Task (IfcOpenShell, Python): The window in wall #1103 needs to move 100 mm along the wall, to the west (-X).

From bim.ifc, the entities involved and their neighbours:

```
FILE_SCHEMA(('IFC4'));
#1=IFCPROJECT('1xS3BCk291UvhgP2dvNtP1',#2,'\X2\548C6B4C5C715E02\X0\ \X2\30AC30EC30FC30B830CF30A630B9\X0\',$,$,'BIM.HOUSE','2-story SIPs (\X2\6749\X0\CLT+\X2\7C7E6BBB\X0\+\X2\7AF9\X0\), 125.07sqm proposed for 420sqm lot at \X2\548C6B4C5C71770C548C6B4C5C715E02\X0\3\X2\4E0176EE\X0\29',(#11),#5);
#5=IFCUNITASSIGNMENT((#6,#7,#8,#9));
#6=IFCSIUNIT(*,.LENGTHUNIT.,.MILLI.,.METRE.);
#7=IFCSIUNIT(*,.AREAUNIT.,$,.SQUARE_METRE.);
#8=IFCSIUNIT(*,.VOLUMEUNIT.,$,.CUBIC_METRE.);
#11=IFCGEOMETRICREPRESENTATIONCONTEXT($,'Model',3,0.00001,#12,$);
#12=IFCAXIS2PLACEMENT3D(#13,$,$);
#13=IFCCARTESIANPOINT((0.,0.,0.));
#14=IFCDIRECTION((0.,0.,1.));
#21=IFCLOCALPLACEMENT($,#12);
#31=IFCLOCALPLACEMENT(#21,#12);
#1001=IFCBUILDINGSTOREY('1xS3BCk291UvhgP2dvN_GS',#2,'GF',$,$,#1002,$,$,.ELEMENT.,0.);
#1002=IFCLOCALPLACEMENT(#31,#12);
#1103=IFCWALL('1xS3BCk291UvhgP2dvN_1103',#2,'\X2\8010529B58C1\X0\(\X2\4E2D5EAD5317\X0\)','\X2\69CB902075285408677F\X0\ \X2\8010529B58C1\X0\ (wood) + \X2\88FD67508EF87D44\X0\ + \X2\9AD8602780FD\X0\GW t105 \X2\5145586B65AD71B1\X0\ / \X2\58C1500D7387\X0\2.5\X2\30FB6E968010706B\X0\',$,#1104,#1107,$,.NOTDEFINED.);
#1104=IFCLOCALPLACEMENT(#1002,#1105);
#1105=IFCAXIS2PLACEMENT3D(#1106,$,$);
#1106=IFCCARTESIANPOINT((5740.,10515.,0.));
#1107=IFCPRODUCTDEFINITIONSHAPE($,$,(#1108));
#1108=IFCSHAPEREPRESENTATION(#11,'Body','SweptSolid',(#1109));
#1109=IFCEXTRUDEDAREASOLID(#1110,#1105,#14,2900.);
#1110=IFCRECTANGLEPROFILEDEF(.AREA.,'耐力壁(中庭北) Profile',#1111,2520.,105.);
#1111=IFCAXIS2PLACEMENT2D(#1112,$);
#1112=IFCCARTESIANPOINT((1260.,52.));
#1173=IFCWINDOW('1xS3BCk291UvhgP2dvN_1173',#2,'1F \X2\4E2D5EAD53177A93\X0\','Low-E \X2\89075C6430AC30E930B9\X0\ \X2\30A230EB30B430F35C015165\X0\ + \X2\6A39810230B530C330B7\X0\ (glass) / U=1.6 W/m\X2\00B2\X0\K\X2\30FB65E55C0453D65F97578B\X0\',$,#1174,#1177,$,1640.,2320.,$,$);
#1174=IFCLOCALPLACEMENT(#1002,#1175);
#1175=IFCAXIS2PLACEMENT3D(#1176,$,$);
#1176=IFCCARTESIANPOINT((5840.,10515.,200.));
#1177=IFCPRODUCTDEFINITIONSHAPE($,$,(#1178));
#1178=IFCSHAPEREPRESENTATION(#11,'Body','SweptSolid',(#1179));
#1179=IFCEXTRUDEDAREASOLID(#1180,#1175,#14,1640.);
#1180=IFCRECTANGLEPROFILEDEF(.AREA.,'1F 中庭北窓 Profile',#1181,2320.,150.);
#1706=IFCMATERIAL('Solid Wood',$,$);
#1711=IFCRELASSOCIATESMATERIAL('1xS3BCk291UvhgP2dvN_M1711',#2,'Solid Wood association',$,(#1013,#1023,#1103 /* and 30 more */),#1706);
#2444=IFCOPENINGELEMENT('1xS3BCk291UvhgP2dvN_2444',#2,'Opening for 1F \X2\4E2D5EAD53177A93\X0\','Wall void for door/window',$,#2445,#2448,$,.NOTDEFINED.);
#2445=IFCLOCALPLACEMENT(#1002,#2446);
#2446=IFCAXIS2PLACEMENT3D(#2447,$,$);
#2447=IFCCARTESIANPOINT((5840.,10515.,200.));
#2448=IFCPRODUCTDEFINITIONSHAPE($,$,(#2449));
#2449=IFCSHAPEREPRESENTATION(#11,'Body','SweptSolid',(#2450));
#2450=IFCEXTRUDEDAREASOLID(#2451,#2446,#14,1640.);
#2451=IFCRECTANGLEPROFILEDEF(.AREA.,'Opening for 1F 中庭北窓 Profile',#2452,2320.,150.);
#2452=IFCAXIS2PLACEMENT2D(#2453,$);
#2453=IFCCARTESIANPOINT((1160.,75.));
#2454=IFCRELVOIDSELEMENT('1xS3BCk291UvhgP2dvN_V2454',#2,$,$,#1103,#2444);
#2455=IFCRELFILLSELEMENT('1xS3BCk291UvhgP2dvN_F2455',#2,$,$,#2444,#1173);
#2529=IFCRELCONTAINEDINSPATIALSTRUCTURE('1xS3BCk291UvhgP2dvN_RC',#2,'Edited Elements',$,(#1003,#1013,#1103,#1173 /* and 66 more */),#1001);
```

```python
import ifcopenshell
import ifcopenshell.api.geometry
import ifcopenshell.util.placement
import ifcopenshell.util.unit

model = ifcopenshell.open("bim.ifc")
unit_scale = ifcopenshell.util.unit.calculate_unit_scale(model)

window = model.by_guid("1xS3BCk291UvhgP2dvN_1173")
opening = window.FillsVoids[0].RelatingOpeningElement
wall = opening.VoidsElements[0].RelatingBuildingElement

wall_matrix = ifcopenshell.util.placement.get_local_placement(wall.ObjectPlacement)
shift = wall_matrix[:3, 0] * -0.1 / unit_scale
before = ifcopenshell.util.placement.get_local_placement(window.ObjectPlacement)[:3, 3].copy()

# The window is not placed relative to its opening, so move both.
for product in (opening, window):
    matrix = ifcopenshell.util.placement.get_local_placement(product.ObjectPlacement)
    matrix[:3, 3] += shift
    ifcopenshell.api.geometry.edit_object_placement(model, product=product, matrix=matrix, is_si=False)

after = ifcopenshell.util.placement.get_local_placement(window.ObjectPlacement)[:3, 3]
print("window moved by", (after - before).round(3) + 0.0)

model.write("bim_updated.ifc")
```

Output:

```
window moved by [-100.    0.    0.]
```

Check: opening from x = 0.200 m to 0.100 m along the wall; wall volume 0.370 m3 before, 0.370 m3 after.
